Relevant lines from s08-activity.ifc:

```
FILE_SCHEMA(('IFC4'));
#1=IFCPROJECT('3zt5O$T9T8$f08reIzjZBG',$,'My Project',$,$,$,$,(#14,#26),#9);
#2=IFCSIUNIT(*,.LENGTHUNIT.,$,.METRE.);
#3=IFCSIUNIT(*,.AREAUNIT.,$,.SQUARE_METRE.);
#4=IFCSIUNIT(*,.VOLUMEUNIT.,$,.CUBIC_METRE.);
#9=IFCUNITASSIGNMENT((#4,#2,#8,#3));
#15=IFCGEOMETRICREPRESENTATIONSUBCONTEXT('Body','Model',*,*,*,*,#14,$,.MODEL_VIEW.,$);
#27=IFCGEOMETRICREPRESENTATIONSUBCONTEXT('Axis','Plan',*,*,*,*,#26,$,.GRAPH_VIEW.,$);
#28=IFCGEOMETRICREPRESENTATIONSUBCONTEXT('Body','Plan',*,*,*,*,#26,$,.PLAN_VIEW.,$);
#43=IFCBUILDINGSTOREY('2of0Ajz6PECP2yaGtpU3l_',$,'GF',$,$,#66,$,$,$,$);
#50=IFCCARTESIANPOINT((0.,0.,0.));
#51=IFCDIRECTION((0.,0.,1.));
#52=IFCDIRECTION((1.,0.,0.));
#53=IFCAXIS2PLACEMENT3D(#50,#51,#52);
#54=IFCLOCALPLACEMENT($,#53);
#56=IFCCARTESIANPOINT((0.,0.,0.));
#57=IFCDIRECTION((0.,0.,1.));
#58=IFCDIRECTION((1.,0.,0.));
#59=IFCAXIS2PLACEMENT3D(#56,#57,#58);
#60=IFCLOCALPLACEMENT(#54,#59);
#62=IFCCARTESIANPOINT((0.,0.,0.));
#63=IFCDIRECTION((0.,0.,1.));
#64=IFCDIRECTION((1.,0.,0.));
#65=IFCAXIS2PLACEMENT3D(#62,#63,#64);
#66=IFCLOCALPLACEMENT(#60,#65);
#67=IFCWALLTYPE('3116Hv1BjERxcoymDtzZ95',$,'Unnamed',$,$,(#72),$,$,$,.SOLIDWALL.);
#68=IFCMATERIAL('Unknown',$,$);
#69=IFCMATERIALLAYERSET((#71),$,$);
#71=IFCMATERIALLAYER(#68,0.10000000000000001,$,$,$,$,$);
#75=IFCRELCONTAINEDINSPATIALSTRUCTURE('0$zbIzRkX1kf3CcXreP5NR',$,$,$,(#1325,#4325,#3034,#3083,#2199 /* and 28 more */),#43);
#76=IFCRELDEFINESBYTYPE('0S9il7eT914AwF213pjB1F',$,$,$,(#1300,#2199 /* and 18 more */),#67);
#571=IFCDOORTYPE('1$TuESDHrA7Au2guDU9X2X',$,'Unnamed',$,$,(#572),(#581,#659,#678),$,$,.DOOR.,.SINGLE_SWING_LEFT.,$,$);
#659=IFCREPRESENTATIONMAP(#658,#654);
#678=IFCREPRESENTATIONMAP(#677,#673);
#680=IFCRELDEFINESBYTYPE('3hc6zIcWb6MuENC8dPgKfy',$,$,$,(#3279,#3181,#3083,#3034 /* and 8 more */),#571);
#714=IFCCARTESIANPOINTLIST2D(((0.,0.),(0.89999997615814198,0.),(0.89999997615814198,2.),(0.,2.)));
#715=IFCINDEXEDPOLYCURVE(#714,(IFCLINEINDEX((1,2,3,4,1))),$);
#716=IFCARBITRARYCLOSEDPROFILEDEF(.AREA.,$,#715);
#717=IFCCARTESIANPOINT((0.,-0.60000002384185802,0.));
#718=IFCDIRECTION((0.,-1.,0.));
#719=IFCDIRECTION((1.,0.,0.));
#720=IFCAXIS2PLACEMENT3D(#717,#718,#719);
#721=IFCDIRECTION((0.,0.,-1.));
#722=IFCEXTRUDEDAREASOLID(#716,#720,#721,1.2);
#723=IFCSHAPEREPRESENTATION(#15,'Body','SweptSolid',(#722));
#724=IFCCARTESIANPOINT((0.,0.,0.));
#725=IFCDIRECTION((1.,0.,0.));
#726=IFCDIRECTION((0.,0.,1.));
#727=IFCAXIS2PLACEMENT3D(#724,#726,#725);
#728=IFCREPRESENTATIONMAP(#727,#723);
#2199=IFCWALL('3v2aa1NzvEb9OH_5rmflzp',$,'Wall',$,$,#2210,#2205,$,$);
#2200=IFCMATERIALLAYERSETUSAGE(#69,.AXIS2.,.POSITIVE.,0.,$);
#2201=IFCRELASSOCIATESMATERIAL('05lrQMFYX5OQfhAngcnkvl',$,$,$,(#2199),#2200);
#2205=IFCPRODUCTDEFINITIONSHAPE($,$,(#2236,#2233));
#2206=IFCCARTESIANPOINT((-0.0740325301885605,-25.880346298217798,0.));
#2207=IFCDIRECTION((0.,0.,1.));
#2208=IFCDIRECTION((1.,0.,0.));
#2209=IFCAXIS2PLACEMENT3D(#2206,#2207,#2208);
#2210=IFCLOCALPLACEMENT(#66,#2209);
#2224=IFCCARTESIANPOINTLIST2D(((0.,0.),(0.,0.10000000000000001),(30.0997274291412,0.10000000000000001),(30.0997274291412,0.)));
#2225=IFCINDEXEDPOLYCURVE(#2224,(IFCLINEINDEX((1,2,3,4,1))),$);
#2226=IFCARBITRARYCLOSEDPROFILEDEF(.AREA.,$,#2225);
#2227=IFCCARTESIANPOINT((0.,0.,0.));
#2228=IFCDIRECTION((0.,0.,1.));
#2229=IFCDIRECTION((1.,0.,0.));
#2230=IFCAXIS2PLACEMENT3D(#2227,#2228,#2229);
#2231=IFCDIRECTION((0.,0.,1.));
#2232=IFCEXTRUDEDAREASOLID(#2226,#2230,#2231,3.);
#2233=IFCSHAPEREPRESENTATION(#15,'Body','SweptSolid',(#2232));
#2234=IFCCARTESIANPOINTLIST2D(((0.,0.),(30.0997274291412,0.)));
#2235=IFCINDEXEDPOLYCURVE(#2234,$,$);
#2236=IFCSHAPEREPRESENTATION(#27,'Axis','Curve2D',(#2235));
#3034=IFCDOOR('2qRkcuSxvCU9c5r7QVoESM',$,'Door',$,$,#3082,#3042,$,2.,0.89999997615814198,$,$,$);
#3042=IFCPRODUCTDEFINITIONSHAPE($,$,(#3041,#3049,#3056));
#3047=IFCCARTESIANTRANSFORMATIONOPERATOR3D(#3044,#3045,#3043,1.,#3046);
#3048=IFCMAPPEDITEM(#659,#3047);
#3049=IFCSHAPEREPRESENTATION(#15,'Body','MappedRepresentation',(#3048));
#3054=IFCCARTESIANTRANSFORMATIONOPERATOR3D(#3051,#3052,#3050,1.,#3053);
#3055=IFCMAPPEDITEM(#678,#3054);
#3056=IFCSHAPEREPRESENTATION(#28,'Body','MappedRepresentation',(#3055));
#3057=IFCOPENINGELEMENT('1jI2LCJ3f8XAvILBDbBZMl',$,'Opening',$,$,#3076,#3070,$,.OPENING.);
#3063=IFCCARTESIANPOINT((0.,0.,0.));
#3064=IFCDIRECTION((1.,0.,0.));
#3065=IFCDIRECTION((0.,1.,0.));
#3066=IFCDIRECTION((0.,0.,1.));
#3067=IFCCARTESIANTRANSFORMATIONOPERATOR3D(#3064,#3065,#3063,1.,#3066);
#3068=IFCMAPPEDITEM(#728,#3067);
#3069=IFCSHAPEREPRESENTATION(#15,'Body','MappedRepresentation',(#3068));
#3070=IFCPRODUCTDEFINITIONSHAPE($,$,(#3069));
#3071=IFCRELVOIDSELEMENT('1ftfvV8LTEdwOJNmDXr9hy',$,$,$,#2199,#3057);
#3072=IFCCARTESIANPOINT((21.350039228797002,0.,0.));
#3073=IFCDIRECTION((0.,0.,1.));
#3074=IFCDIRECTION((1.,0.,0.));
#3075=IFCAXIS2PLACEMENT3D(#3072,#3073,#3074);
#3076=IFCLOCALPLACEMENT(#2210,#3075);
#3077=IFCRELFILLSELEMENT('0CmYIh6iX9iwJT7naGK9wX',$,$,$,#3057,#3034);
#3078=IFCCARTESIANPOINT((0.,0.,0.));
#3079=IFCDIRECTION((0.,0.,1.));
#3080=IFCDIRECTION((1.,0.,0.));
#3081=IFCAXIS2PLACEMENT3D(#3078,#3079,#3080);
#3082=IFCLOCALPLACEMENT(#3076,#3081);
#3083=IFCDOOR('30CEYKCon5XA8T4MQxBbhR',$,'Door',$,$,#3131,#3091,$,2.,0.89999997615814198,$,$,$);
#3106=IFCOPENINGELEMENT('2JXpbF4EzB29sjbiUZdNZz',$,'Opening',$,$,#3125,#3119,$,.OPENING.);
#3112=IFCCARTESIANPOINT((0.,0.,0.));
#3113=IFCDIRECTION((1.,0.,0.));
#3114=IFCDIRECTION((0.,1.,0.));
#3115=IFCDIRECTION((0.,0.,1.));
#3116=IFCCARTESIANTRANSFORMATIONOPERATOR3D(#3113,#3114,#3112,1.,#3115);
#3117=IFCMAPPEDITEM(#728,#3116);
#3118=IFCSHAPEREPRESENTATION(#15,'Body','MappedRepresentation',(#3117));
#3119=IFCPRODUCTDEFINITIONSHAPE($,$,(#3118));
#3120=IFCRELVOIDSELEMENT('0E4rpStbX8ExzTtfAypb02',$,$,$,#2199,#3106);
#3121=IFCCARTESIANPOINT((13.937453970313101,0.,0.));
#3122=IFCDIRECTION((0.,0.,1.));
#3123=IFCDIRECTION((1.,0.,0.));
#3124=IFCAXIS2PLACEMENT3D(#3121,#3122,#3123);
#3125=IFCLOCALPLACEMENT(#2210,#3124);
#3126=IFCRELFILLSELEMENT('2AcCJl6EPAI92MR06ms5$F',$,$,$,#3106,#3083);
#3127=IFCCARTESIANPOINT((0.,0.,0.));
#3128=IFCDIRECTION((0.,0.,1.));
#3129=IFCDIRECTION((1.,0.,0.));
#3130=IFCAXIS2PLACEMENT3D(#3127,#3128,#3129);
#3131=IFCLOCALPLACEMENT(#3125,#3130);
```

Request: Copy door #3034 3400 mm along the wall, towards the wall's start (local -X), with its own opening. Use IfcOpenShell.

```python
import ifcopenshell
import ifcopenshell.api.feature
import ifcopenshell.api.geometry
import ifcopenshell.api.root
import ifcopenshell.geom
import ifcopenshell.util.element
import ifcopenshell.util.placement
import ifcopenshell.util.shape

model = ifcopenshell.open("s08-activity.ifc")
settings = ifcopenshell.geom.settings()


def volume(element):
    """Net volume in cubic metres, openings subtracted."""
    shape = ifcopenshell.geom.create_shape(settings, element)
    return ifcopenshell.util.shape.get_volume(shape.geometry)


door = model.by_guid("2qRkcuSxvCU9c5r7QVoESM")
opening = door.FillsVoids[0].RelatingOpeningElement
wall = opening.VoidsElements[0].RelatingBuildingElement
before = volume(wall)
shift = ifcopenshell.util.placement.get_local_placement(wall.ObjectPlacement)[:3, 0] * -3.4

# copy_class copies the void relationship, type, container and properties, but no geometry.
new_opening = ifcopenshell.api.root.copy_class(model, product=opening)
new_opening.Representation = ifcopenshell.util.element.copy_deep(
    model, opening.Representation, exclude=["IfcGeometricRepresentationContext", "IfcRepresentationMap"]
)
new_door = ifcopenshell.api.root.copy_class(model, product=door)
new_door.Representation = ifcopenshell.util.element.copy_deep(
    model, door.Representation, exclude=["IfcGeometricRepresentationContext", "IfcRepresentationMap"]
)
ifcopenshell.api.feature.add_filling(model, opening=new_opening, element=new_door)

for old, new in ((opening, new_opening), (door, new_door)):
    matrix = ifcopenshell.util.placement.get_local_placement(old.ObjectPlacement)
    matrix[:3, 3] += shift
    ifcopenshell.api.geometry.edit_object_placement(model, product=new, matrix=matrix, is_si=False)

after = volume(wall)

print(f"wall volume {before:.3f} -> {after:.3f} m3")

model.write("s08-activity-out.ifc")
```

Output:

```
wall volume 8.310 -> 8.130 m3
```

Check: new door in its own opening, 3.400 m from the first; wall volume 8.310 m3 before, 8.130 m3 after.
